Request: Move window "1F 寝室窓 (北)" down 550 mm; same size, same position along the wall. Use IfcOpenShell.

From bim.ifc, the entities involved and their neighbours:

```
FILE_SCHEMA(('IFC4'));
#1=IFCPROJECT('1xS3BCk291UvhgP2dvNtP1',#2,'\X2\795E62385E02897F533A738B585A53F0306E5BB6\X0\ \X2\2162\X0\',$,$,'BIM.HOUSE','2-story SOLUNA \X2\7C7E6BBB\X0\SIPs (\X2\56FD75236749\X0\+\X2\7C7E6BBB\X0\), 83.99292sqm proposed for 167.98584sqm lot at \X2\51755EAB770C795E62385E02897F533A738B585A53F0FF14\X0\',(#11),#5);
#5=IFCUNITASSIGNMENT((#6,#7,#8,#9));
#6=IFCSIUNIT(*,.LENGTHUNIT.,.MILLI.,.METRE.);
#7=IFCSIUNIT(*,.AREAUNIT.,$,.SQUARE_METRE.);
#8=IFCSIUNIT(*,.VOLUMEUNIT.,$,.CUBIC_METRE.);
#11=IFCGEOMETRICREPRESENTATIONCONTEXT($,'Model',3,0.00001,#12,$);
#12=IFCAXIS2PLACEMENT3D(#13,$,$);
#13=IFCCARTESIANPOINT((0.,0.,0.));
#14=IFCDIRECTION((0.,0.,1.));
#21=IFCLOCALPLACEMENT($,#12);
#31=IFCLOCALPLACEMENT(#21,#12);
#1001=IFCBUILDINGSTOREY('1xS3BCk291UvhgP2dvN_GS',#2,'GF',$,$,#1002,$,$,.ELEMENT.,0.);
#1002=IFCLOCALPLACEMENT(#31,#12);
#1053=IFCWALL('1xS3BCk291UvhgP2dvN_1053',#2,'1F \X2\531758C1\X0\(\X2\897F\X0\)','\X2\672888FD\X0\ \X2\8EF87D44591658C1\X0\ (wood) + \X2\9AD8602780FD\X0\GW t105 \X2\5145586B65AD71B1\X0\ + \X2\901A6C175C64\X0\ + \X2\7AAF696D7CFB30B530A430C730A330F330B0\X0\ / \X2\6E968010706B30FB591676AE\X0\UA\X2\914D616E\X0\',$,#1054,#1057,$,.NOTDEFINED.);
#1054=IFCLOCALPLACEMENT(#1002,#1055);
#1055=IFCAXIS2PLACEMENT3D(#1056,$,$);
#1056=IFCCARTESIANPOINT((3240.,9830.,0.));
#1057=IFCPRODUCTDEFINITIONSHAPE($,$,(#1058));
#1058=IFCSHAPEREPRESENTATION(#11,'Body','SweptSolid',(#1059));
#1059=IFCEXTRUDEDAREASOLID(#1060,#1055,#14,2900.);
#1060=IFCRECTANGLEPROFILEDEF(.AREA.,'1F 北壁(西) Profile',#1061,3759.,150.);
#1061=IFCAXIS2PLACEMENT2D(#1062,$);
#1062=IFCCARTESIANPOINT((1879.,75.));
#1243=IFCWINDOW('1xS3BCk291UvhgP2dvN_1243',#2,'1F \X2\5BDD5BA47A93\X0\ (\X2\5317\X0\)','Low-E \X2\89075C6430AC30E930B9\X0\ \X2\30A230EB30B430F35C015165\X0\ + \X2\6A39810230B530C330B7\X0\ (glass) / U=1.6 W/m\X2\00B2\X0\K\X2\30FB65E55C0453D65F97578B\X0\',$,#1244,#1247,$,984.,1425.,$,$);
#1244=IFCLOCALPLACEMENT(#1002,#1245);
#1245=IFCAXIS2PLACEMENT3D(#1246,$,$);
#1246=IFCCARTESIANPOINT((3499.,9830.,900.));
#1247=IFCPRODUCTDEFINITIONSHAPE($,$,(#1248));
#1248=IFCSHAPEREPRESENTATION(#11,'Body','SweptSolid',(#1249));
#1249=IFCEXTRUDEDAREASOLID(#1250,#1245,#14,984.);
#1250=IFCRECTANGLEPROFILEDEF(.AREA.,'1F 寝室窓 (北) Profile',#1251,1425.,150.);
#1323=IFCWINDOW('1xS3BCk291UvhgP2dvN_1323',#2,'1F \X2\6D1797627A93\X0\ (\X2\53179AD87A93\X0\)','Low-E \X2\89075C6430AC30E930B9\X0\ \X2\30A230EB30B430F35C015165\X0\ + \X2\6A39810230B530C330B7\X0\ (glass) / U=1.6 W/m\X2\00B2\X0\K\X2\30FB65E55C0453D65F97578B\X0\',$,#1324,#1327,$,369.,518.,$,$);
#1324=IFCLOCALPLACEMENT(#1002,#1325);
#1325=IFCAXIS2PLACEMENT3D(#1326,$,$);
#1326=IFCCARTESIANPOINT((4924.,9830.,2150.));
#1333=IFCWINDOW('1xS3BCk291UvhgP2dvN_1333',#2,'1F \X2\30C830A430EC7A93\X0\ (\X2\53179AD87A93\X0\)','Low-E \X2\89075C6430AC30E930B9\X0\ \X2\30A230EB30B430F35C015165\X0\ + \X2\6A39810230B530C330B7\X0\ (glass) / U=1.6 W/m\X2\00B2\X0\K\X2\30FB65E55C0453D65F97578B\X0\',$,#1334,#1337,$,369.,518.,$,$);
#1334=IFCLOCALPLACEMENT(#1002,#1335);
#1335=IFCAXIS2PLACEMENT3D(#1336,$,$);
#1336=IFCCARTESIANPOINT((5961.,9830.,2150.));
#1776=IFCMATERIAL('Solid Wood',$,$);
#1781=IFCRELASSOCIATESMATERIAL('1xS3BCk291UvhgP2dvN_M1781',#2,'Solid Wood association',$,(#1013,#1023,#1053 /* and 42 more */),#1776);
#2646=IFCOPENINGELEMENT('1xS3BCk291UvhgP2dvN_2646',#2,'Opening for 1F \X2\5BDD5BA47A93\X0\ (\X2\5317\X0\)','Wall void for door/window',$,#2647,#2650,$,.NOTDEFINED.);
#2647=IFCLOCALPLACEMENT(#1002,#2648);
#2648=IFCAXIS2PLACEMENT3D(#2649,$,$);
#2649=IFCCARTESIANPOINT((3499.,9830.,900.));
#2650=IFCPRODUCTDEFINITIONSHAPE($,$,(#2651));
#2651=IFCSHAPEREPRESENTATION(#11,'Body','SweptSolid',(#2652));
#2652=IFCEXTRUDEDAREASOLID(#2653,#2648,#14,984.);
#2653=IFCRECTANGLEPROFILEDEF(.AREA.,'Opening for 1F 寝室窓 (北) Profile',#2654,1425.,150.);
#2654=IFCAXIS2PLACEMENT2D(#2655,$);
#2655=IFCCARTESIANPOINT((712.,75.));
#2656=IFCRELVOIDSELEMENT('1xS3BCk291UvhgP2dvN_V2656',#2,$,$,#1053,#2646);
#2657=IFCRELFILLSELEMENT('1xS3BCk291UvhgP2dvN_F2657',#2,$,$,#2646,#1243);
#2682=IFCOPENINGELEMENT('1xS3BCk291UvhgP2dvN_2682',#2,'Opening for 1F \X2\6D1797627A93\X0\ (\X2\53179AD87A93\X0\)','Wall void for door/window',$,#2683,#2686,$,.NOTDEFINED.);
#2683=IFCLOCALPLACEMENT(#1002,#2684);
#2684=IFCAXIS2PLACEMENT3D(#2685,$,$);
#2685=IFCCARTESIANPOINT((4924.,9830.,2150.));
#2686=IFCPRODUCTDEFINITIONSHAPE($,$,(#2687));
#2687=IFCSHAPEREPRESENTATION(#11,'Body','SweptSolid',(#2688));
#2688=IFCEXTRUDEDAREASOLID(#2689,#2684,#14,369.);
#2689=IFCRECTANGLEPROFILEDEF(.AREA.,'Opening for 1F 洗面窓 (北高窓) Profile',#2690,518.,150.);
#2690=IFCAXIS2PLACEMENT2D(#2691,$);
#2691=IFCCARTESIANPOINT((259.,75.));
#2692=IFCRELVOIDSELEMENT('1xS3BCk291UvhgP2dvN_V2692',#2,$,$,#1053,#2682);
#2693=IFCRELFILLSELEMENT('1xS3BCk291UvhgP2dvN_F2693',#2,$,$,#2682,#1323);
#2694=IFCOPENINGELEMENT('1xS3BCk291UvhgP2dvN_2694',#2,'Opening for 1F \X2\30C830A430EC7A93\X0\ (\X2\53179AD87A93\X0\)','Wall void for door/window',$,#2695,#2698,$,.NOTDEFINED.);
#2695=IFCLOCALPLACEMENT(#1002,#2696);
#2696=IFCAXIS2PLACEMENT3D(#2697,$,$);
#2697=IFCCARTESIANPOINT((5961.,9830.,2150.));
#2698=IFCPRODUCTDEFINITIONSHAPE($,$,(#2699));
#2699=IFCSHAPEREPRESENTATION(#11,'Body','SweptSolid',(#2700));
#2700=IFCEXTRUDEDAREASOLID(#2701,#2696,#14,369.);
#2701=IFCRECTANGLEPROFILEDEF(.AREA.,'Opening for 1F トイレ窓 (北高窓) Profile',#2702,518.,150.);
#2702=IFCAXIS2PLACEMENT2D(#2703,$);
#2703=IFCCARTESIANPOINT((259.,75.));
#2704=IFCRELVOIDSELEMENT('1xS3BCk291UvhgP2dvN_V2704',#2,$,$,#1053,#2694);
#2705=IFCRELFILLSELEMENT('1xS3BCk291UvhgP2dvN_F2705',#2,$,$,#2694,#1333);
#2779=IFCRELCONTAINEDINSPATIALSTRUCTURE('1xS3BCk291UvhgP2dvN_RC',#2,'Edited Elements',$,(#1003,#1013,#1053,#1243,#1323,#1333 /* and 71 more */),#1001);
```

```python
import numpy as np
import ifcopenshell
import ifcopenshell.api.geometry
import ifcopenshell.util.placement
import ifcopenshell.util.unit

model = ifcopenshell.open("bim.ifc")
unit_scale = ifcopenshell.util.unit.calculate_unit_scale(model)

window = model.by_guid("1xS3BCk291UvhgP2dvN_1243")
opening = window.FillsVoids[0].RelatingOpeningElement
dz = -0.55 / unit_scale

shift = np.array([0.0, 0.0, dz])
# The window is not placed relative to its opening, so move both.
for product in (opening, window):
    matrix = ifcopenshell.util.placement.get_local_placement(product.ObjectPlacement)
    matrix[:3, 3] += shift
    ifcopenshell.api.geometry.edit_object_placement(model, product=product, matrix=matrix, is_si=False)

print(f"moved by {dz * unit_scale:+.3f} m")

model.write("bim_updated.ifc")
```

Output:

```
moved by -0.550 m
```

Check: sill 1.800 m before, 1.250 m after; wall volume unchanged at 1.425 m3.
